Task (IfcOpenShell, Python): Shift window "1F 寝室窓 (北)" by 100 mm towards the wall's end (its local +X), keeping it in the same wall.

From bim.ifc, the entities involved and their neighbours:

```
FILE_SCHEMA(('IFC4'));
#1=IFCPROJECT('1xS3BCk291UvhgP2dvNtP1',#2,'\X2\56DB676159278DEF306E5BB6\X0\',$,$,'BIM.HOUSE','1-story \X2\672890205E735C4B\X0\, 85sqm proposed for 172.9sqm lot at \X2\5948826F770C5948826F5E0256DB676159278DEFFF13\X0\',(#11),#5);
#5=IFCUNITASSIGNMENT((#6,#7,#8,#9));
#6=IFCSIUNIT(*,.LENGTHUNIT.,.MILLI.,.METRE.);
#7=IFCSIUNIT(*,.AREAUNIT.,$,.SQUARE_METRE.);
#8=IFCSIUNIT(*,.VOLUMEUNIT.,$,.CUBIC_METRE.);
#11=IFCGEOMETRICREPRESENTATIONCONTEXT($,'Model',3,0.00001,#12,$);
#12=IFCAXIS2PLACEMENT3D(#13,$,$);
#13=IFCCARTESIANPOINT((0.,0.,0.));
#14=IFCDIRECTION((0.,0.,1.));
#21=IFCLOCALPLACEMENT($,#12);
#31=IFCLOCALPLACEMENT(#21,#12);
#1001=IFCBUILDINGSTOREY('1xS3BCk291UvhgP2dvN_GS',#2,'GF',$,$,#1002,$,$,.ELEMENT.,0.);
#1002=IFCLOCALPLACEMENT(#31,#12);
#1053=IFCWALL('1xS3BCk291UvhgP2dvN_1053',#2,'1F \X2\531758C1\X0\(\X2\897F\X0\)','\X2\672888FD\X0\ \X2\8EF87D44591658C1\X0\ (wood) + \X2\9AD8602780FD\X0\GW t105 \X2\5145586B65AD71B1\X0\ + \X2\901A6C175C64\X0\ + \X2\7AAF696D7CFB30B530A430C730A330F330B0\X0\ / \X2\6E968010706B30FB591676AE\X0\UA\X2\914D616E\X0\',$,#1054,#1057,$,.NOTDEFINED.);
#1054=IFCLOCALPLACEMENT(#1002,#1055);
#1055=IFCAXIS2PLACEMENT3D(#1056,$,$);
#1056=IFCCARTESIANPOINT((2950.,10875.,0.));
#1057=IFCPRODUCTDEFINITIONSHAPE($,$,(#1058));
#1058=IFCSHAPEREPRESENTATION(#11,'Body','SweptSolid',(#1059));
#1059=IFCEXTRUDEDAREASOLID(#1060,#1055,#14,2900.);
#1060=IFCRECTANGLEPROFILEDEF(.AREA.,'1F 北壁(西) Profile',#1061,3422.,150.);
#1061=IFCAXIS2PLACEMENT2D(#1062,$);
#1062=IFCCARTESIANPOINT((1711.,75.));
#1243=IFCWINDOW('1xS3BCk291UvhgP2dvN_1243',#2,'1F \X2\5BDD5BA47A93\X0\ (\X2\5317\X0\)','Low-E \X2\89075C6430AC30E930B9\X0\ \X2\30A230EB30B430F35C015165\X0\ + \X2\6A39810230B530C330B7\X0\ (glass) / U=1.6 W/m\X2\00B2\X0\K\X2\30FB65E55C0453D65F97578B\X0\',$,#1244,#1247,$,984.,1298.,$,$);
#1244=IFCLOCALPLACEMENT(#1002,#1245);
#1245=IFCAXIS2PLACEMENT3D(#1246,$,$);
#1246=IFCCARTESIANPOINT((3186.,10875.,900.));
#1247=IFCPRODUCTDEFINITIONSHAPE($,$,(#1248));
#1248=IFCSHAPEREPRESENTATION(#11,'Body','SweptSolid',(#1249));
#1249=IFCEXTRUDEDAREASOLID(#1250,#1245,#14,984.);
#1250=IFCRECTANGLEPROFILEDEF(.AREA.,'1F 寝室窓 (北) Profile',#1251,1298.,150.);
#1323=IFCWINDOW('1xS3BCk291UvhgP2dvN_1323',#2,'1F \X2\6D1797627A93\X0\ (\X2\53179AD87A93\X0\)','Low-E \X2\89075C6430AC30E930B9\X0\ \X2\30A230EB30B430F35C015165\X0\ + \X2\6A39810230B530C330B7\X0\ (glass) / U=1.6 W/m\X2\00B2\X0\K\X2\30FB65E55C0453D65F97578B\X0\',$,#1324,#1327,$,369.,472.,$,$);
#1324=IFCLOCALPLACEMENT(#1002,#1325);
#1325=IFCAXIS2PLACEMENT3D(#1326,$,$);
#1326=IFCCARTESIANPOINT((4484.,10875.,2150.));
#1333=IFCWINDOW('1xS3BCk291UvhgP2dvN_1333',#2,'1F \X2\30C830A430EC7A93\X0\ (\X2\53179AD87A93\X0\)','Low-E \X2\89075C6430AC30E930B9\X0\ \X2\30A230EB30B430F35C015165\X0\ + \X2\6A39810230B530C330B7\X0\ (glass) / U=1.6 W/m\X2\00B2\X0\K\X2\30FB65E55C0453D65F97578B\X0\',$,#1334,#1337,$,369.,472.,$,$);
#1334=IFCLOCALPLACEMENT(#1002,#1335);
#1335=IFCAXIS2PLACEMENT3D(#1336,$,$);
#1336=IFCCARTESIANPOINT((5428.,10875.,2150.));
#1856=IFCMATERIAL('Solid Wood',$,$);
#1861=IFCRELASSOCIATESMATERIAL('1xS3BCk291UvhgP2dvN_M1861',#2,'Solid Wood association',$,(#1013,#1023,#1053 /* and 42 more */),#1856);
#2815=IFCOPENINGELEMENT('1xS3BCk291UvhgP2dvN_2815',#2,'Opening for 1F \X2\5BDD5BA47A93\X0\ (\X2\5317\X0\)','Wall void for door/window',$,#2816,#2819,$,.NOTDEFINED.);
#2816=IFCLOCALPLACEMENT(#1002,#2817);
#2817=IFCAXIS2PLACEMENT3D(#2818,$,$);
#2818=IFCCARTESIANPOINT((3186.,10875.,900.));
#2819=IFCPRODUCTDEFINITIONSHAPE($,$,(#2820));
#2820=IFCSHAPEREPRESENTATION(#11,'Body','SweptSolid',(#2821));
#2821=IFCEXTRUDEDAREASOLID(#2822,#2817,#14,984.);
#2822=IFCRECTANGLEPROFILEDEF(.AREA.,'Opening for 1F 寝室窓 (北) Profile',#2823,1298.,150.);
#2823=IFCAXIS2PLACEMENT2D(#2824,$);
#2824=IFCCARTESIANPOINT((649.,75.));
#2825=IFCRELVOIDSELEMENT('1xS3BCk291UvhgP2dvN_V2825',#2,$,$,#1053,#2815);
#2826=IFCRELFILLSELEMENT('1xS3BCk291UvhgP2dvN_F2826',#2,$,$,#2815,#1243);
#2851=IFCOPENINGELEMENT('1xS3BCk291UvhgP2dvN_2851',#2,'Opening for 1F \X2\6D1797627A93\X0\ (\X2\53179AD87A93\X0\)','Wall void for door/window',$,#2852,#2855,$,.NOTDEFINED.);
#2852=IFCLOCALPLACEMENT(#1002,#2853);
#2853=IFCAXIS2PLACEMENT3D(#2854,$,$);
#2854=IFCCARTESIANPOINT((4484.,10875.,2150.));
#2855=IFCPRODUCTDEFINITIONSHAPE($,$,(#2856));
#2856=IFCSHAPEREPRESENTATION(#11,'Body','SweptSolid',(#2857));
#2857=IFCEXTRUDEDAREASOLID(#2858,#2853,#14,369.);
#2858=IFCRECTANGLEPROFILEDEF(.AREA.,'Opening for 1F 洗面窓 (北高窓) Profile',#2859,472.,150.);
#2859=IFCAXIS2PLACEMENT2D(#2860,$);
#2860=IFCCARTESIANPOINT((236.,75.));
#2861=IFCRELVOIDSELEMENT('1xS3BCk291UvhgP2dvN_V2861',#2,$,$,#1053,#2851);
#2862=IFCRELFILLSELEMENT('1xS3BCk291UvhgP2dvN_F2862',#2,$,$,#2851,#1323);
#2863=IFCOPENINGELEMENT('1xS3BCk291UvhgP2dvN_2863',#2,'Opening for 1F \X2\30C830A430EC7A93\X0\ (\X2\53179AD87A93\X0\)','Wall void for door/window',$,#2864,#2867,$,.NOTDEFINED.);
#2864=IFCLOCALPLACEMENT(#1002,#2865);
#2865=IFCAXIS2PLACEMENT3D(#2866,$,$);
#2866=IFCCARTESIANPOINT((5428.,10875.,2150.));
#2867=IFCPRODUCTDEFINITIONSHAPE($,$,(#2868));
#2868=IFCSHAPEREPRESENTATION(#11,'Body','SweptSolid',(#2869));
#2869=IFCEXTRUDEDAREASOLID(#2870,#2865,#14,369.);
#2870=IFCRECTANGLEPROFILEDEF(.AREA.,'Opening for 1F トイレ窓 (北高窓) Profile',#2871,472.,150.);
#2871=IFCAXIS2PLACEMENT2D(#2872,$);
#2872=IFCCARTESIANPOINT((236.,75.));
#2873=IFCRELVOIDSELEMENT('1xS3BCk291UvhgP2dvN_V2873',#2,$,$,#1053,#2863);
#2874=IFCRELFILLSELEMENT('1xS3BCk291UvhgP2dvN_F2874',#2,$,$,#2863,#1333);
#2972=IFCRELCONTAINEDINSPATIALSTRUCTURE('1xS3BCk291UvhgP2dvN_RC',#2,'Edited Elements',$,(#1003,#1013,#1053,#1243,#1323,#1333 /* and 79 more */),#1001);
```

```python
import ifcopenshell
import ifcopenshell.api.geometry
import ifcopenshell.util.placement
import ifcopenshell.util.unit

model = ifcopenshell.open("bim.ifc")
unit_scale = ifcopenshell.util.unit.calculate_unit_scale(model)

window = model.by_guid("1xS3BCk291UvhgP2dvN_1243")
opening = window.FillsVoids[0].RelatingOpeningElement
wall = opening.VoidsElements[0].RelatingBuildingElement

wall_matrix = ifcopenshell.util.placement.get_local_placement(wall.ObjectPlacement)
shift = wall_matrix[:3, 0] * 0.1 / unit_scale
before = ifcopenshell.util.placement.get_local_placement(window.ObjectPlacement)[:3, 3].copy()

# The window is not placed relative to its opening, so move both.
for product in (opening, window):
    matrix = ifcopenshell.util.placement.get_local_placement(product.ObjectPlacement)
    matrix[:3, 3] += shift
    ifcopenshell.api.geometry.edit_object_placement(model, product=product, matrix=matrix, is_si=False)

after = ifcopenshell.util.placement.get_local_placement(window.ObjectPlacement)[:3, 3]
print("window moved by", (after - before).round(3) + 0.0)

model.write("bim_updated.ifc")
```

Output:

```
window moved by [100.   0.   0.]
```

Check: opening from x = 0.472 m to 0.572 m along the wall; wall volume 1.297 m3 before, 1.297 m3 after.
